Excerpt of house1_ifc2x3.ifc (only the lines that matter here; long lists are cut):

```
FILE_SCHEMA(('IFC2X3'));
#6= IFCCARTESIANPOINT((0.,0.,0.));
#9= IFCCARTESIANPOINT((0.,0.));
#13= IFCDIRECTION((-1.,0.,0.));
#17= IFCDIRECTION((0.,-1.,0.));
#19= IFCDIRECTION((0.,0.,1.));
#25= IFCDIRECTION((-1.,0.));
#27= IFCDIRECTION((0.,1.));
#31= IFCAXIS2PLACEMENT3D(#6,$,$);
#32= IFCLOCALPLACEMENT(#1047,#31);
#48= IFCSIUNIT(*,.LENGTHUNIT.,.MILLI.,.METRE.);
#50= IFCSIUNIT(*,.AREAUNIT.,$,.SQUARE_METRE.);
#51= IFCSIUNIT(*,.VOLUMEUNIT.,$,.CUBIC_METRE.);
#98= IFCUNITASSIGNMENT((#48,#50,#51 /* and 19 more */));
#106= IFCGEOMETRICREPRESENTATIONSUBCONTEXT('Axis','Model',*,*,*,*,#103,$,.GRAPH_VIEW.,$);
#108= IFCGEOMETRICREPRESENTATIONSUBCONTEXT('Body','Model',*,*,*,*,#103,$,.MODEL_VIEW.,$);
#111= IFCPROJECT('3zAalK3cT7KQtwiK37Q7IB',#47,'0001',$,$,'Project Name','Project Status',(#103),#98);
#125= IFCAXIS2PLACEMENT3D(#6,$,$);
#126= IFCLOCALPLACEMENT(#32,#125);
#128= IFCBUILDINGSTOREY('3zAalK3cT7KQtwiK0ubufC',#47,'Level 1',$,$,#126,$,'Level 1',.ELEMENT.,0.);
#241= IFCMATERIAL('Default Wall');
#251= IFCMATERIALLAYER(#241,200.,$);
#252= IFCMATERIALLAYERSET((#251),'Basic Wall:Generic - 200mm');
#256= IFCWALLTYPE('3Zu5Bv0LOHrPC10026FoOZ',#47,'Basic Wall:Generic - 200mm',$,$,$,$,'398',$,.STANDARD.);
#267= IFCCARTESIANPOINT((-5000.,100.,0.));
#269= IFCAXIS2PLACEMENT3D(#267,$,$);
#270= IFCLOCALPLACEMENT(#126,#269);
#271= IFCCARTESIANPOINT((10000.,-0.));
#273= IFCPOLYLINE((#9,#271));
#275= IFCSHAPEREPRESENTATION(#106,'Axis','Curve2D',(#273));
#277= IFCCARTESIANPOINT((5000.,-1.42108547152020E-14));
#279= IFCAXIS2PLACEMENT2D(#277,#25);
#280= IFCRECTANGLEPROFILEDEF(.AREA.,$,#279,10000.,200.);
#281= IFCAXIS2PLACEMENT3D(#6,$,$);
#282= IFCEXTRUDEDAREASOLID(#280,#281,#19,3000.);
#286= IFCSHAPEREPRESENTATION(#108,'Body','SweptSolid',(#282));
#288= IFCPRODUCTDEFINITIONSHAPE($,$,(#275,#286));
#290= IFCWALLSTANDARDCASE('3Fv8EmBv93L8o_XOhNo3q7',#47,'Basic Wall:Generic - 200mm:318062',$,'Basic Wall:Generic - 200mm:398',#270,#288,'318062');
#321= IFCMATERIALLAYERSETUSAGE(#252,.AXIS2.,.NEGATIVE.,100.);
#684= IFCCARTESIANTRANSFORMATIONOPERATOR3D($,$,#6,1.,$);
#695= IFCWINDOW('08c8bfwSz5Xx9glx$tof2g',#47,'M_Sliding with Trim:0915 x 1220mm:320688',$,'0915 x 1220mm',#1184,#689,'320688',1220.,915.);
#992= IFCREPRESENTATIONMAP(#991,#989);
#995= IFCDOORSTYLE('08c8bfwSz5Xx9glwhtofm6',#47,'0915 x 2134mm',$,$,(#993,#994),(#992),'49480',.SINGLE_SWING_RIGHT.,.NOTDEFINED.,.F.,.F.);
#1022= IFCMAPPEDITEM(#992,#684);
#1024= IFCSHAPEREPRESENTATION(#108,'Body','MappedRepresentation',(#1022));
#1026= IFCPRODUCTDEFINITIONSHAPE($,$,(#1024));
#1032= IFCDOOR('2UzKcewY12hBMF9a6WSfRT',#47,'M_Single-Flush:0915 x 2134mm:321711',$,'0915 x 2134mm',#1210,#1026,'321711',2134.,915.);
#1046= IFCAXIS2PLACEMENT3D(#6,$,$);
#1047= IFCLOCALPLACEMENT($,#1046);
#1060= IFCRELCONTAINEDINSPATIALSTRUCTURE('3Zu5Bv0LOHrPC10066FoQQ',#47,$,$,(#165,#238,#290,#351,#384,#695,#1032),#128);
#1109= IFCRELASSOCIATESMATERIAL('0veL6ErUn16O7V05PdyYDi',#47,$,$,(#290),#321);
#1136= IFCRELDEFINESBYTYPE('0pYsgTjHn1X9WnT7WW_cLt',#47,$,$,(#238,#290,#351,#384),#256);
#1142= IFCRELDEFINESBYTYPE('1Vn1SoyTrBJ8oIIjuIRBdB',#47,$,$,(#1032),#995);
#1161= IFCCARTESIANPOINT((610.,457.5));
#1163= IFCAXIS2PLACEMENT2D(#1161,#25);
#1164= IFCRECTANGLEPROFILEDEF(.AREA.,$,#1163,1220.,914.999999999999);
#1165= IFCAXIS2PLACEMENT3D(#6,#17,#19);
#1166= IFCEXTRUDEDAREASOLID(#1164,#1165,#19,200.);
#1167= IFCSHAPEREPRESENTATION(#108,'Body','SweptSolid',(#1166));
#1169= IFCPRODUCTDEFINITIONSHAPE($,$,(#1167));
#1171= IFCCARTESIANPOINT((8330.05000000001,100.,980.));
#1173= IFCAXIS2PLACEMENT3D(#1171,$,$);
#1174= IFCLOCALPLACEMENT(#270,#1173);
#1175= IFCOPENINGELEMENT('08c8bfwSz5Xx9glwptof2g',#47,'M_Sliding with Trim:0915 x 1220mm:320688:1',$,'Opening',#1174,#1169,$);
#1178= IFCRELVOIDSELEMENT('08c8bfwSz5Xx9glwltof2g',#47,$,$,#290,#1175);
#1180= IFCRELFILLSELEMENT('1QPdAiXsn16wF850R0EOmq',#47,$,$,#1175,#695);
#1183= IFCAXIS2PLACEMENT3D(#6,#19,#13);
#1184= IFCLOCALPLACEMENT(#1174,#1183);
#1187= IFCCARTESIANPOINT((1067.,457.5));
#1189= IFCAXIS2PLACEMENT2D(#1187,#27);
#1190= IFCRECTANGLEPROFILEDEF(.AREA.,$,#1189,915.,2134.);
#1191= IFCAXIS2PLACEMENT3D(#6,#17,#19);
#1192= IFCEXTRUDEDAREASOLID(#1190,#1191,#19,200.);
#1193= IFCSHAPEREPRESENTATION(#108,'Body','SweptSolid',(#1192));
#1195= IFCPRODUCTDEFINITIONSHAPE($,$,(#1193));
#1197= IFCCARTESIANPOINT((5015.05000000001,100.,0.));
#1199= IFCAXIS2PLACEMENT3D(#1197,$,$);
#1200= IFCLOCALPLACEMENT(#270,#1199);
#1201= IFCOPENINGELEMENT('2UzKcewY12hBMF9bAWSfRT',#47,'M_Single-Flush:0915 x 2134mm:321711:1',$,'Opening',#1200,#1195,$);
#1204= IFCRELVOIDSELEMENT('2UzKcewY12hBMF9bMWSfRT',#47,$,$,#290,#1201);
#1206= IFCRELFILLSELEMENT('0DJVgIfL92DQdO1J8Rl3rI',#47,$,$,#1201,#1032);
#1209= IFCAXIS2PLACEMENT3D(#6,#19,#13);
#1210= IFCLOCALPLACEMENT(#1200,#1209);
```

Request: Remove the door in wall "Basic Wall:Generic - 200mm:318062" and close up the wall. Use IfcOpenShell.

```python
import ifcopenshell
import ifcopenshell.api.feature
import ifcopenshell.api.root
import ifcopenshell.geom
import ifcopenshell.util.shape

model = ifcopenshell.open("house1_ifc2x3.ifc")
settings = ifcopenshell.geom.settings()


def volume(element):
    """Net volume in cubic metres, openings subtracted."""
    shape = ifcopenshell.geom.create_shape(settings, element)
    return ifcopenshell.util.shape.get_volume(shape.geometry)


door = model.by_guid("2UzKcewY12hBMF9a6WSfRT")
opening = door.FillsVoids[0].RelatingOpeningElement
wall = opening.VoidsElements[0].RelatingBuildingElement
before = volume(wall)

ifcopenshell.api.root.remove_product(model, product=door)
ifcopenshell.api.feature.remove_feature(model, feature=opening)

after = volume(wall)

print(f"wall volume {before:.3f} -> {after:.3f} m3")

model.write("house1_ifc2x3_v2.ifc")
```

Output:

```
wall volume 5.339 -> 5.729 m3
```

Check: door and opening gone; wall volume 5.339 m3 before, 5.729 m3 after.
